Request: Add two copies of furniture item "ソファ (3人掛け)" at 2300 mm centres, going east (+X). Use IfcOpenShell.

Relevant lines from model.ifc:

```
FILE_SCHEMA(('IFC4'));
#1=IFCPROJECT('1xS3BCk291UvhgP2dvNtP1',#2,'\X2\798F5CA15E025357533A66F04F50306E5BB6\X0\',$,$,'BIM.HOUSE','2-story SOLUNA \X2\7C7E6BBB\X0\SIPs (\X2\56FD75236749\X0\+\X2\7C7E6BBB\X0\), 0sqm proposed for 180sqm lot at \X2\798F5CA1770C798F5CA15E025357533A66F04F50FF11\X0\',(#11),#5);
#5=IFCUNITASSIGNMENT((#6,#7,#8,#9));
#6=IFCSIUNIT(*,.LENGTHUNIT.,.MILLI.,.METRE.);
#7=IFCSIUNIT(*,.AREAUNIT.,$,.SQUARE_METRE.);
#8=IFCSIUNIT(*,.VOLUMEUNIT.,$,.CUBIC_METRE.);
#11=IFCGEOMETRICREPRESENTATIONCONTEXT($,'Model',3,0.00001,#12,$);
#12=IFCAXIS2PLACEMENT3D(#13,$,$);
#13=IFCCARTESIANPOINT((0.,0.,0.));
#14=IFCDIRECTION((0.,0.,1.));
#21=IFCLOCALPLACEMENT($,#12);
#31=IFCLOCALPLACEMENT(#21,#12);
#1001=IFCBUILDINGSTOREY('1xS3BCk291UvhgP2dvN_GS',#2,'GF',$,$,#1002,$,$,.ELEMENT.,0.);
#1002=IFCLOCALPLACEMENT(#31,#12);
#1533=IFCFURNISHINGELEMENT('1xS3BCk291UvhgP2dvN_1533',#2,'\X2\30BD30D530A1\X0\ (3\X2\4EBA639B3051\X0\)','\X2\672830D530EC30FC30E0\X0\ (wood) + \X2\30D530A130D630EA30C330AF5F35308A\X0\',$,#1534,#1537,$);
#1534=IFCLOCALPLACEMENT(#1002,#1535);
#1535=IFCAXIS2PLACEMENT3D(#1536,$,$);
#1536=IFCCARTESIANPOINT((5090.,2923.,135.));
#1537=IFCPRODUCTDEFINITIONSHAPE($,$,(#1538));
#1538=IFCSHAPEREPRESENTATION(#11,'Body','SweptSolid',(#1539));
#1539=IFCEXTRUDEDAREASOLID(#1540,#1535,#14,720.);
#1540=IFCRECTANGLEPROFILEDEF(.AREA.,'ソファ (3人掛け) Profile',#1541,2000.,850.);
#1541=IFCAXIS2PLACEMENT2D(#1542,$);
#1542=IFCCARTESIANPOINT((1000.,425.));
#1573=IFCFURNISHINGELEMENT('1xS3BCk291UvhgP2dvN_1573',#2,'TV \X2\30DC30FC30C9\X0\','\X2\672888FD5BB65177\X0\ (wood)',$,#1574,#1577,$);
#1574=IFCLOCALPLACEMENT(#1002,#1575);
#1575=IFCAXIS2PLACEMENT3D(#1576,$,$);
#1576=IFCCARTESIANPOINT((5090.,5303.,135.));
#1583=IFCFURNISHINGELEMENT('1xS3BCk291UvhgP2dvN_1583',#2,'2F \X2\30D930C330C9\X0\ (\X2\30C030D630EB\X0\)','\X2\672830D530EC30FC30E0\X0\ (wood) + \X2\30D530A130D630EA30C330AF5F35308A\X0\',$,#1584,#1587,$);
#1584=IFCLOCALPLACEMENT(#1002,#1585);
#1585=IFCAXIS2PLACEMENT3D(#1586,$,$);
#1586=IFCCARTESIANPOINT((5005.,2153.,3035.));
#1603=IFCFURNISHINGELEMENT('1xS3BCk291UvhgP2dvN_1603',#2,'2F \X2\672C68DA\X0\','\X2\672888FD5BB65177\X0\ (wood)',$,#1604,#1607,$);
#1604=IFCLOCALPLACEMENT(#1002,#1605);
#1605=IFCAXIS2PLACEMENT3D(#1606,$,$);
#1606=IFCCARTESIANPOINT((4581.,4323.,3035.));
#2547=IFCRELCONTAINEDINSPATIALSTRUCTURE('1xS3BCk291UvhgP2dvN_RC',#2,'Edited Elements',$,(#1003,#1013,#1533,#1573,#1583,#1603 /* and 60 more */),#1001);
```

```python
import numpy as np
import ifcopenshell
import ifcopenshell.api.geometry
import ifcopenshell.api.root
import ifcopenshell.util.element
import ifcopenshell.util.placement
import ifcopenshell.util.unit

model = ifcopenshell.open("model.ifc")
unit_scale = ifcopenshell.util.unit.calculate_unit_scale(model)


def reuse_history(source, copy):
    """copy_class also copies each property set's owner history, people and application; keep the originals."""
    for rel in copy.IsDefinedBy:
        if rel.is_a("IfcRelDefinesByProperties") and (history := rel.RelatingPropertyDefinition.OwnerHistory):
            rel.RelatingPropertyDefinition.OwnerHistory = source.OwnerHistory
            ifcopenshell.util.element.remove_deep2(model, history)


source = model.by_guid("1xS3BCk291UvhgP2dvN_1533")
base = ifcopenshell.util.placement.get_local_placement(source.ObjectPlacement)
step = np.array([1.0, 0.0, 0.0]) * 2.3 / unit_scale

for i in range(1, 3):
    copy = ifcopenshell.api.root.copy_class(model, product=source)
    copy.Representation = ifcopenshell.util.element.copy_deep(
        model, source.Representation, exclude=["IfcGeometricRepresentationContext", "IfcRepresentationMap"]
    )
    reuse_history(source, copy)
    matrix = base.copy()
    matrix[:3, 3] += i * step
    print("added at", matrix[:3, 3].round(3) + 0.0)
    ifcopenshell.api.geometry.edit_object_placement(model, product=copy, matrix=matrix, is_si=False)

model.write("model_v2.ifc")
```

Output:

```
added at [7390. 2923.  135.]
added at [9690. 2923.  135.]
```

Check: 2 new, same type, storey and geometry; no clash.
